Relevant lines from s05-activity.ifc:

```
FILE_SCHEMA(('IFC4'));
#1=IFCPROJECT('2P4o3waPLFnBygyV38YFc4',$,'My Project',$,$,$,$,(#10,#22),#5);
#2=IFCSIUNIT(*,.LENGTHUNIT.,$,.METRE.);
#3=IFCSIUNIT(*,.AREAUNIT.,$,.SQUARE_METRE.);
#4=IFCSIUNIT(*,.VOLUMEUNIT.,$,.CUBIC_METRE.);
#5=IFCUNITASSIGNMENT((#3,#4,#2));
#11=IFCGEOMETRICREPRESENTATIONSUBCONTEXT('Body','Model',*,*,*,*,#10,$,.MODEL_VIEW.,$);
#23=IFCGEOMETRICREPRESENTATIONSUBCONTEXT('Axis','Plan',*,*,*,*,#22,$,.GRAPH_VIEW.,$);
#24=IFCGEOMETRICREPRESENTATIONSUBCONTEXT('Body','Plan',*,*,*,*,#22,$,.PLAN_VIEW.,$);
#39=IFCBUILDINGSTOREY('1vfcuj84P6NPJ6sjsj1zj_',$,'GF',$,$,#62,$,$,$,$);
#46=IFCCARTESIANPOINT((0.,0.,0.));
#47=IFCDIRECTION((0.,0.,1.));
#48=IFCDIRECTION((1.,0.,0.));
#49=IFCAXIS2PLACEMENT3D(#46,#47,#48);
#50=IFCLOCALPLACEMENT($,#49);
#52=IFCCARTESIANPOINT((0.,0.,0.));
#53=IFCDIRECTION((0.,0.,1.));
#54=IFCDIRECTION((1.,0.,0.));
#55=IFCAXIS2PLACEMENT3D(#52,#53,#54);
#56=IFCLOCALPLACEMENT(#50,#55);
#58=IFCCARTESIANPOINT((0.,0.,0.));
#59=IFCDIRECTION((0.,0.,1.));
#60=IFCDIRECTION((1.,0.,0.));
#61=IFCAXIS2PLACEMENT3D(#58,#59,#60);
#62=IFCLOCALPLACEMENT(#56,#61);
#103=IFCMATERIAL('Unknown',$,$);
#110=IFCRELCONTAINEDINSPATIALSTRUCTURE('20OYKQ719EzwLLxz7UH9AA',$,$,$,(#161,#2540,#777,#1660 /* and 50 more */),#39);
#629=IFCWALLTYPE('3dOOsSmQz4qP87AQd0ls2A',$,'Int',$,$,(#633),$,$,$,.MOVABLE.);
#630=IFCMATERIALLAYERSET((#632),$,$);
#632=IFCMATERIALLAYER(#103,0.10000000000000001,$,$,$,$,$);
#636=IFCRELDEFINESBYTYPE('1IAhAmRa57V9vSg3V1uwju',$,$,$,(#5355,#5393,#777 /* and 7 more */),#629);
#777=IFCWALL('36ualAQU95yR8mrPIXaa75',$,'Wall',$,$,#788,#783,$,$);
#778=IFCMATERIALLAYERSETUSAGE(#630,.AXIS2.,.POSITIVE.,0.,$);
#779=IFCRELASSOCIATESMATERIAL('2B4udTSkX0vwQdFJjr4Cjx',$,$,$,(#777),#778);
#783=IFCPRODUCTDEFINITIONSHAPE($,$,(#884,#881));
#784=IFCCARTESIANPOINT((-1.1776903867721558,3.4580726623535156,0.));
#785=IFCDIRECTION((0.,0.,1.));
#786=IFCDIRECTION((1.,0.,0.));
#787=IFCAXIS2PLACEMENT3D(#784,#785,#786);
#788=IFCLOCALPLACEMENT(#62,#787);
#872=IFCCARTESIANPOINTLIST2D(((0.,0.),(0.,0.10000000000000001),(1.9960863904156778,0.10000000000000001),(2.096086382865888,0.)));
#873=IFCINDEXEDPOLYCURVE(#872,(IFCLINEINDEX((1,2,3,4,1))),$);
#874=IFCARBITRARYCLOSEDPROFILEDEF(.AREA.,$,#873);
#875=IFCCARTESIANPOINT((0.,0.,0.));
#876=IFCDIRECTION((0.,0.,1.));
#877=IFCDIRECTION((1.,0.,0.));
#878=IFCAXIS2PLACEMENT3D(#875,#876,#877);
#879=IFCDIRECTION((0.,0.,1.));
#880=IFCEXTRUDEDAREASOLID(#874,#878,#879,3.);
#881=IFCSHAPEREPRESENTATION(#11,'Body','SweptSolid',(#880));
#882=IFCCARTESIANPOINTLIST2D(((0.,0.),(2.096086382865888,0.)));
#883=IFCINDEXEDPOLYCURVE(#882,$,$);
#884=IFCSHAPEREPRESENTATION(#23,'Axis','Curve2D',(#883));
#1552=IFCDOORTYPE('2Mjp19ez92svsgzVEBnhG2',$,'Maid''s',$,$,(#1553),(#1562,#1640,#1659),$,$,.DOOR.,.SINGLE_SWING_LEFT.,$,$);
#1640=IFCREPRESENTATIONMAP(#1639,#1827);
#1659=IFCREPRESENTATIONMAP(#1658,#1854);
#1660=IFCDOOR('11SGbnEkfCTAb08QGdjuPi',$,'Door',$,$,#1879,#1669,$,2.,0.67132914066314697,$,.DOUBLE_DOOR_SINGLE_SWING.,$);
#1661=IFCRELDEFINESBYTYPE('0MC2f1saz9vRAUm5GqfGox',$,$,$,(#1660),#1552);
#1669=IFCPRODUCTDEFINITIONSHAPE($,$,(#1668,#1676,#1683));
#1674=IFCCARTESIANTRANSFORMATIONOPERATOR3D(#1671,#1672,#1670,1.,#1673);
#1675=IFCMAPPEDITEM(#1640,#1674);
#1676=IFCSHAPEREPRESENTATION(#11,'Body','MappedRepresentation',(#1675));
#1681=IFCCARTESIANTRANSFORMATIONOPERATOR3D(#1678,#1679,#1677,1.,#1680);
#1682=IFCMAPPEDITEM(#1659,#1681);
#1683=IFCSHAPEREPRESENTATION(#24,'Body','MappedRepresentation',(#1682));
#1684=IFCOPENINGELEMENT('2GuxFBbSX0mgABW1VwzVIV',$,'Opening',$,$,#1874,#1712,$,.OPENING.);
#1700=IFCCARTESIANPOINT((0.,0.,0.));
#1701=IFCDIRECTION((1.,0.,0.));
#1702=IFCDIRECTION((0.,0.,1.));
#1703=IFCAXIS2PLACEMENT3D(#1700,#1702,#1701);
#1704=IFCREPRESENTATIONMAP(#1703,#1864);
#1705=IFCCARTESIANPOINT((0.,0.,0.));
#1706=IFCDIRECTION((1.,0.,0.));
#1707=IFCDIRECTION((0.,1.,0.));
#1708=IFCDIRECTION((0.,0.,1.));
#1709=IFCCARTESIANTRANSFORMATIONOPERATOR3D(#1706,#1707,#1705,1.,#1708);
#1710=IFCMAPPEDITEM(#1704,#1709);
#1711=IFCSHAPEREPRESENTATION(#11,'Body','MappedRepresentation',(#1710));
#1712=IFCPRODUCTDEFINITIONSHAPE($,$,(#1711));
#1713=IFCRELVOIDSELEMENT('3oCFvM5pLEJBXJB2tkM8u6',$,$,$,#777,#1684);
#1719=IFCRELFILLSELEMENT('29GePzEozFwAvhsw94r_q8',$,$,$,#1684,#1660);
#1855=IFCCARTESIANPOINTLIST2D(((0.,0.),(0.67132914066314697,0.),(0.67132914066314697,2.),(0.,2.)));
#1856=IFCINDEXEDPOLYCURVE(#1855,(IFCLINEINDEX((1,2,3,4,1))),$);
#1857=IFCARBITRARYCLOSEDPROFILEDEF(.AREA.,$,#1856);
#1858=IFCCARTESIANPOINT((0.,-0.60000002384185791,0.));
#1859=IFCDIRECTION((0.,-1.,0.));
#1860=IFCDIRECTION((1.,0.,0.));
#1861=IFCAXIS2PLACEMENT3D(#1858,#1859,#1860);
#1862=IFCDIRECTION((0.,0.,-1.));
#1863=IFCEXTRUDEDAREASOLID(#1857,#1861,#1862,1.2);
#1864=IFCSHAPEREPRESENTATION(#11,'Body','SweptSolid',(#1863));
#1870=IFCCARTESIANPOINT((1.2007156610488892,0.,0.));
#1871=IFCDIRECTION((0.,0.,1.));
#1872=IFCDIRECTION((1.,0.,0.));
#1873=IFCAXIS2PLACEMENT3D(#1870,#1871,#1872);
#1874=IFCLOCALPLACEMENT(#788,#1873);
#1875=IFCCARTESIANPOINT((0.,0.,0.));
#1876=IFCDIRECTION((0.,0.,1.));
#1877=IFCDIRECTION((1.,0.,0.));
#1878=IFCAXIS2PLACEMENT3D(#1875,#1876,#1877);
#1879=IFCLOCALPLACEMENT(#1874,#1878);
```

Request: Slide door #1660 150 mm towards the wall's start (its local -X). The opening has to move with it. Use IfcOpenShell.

```python
import ifcopenshell
import ifcopenshell.api.geometry
import ifcopenshell.util.placement

model = ifcopenshell.open("s05-activity.ifc")

door = model.by_guid("11SGbnEkfCTAb08QGdjuPi")
opening = door.FillsVoids[0].RelatingOpeningElement
wall = opening.VoidsElements[0].RelatingBuildingElement

wall_matrix = ifcopenshell.util.placement.get_local_placement(wall.ObjectPlacement)
shift = wall_matrix[:3, 0] * -0.15
before = ifcopenshell.util.placement.get_local_placement(door.ObjectPlacement)[:3, 3].copy()

# The door is placed relative to its opening, so it follows when the opening moves.
matrix = ifcopenshell.util.placement.get_local_placement(opening.ObjectPlacement)
matrix[:3, 3] += shift
ifcopenshell.api.geometry.edit_object_placement(
    model, product=opening, matrix=matrix, is_si=False, should_transform_children=True
)

after = ifcopenshell.util.placement.get_local_placement(door.ObjectPlacement)[:3, 3]
print("door moved by", (after - before).round(3) + 0.0)

model.write("s05-activity_updated.ifc")
```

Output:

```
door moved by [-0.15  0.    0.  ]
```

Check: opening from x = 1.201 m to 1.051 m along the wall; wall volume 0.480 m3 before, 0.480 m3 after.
